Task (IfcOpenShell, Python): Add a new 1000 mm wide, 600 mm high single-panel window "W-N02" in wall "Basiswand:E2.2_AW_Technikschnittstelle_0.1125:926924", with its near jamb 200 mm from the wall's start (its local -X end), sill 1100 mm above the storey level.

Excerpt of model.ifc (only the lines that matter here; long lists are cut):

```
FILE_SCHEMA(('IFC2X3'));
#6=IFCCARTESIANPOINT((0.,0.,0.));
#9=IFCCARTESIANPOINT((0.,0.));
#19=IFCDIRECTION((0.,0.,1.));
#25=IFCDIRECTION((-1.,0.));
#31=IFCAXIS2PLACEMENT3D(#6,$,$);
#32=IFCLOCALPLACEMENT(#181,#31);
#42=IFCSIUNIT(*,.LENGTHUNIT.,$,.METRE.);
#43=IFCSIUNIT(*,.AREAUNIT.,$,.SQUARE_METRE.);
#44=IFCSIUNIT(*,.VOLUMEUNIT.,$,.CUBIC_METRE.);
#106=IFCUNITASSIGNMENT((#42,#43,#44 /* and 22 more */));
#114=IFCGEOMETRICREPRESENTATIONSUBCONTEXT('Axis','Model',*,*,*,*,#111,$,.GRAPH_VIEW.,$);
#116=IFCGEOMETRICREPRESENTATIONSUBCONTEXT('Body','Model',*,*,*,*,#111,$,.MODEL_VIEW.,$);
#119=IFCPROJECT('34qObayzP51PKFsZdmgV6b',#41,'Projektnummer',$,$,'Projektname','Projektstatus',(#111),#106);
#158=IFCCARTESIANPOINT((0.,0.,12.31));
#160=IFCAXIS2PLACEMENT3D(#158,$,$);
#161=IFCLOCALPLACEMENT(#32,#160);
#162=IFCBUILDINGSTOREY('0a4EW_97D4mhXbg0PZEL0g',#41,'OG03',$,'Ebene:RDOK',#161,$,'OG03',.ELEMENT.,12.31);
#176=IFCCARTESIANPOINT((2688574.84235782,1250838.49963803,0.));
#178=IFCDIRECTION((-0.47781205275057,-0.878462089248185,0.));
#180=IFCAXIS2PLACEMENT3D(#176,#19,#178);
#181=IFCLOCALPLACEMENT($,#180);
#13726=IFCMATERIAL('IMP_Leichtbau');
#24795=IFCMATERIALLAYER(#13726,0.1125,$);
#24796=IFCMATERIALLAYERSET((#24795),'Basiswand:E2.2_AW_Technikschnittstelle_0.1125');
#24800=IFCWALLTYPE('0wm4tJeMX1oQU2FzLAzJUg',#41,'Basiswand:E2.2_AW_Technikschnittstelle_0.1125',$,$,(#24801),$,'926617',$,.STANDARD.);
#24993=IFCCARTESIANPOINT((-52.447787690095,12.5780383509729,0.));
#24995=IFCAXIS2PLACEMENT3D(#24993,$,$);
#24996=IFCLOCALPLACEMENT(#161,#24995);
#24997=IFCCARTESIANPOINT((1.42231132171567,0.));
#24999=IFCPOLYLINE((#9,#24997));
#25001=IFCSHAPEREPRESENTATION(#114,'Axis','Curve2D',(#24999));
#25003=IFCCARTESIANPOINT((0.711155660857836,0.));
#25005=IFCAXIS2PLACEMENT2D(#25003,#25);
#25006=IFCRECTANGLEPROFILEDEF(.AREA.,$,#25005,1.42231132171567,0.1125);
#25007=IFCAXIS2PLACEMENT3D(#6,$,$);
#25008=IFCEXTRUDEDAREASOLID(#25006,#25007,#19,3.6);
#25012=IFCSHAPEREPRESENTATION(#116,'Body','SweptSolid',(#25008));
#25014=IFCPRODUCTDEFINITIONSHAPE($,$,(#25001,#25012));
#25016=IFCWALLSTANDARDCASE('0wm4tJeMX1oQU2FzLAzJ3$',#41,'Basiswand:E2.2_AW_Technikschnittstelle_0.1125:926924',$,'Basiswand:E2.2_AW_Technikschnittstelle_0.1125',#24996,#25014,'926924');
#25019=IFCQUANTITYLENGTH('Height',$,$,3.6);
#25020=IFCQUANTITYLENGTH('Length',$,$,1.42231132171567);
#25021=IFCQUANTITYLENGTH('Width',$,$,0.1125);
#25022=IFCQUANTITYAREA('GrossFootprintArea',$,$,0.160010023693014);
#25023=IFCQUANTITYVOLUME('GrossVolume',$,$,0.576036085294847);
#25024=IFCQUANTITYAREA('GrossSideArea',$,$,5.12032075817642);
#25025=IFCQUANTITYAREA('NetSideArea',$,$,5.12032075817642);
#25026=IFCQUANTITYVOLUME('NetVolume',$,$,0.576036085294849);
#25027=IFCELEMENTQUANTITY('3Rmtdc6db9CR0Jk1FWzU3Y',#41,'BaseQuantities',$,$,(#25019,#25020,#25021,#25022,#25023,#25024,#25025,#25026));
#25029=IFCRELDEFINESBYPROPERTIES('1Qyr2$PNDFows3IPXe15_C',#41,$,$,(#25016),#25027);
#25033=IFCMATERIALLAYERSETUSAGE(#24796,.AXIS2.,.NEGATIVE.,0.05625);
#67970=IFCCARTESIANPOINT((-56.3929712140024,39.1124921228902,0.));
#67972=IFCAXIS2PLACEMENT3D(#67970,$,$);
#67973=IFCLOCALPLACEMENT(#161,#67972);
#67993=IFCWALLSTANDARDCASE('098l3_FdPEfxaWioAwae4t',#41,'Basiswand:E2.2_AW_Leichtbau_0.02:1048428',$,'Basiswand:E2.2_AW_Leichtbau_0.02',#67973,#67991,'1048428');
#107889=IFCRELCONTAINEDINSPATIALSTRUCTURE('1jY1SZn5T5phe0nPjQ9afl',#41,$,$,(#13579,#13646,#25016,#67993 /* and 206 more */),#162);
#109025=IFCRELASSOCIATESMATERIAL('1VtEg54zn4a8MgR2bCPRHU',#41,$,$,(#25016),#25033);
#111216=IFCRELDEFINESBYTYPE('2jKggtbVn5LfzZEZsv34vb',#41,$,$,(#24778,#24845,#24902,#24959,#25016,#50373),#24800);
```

```python
import numpy as np
import ifcopenshell
import ifcopenshell.api.feature
import ifcopenshell.api.geometry
import ifcopenshell.api.pset
import ifcopenshell.api.root
import ifcopenshell.api.spatial
import ifcopenshell.api.type
import ifcopenshell.geom
import ifcopenshell.util.element
import ifcopenshell.util.placement
import ifcopenshell.util.representation
import ifcopenshell.util.shape
import ifcopenshell.util.unit

model = ifcopenshell.open("model.ifc")
unit_scale = ifcopenshell.util.unit.calculate_unit_scale(model)
area_scale = ifcopenshell.util.unit.calculate_unit_scale(model, "AREAUNIT")
volume_scale = ifcopenshell.util.unit.calculate_unit_scale(model, "VOLUMEUNIT")
settings = ifcopenshell.geom.settings()


def volume(element):
    """Net volume in cubic metres, openings subtracted."""
    shape = ifcopenshell.geom.create_shape(settings, element)
    return ifcopenshell.util.shape.get_volume(shape.geometry)


wall = model.by_guid("0wm4tJeMX1oQU2FzLAzJ3$")
storey = ifcopenshell.util.element.get_container(wall, ifc_class="IfcBuildingStorey")
context = ifcopenshell.util.representation.get_context(model, "Model", "Body", "MODEL_VIEW")
before = volume(wall)

width, height, from_end, sill = 1, 0.6, 0.2, 1.1  # metres

# The wall runs along its own X axis, and the end named is its -X end.
wall_shape = ifcopenshell.geom.create_shape(settings, wall)
x, y, z = ifcopenshell.util.shape.get_vertices(wall_shape.geometry).T
start = x.min() + from_end
face, thickness = float(y.min()), float(y.max() - y.min())
wall_matrix = ifcopenshell.util.placement.get_local_placement(wall.ObjectPlacement)
level = ifcopenshell.util.placement.get_local_placement(storey.ObjectPlacement)[2, 3]


def in_wall(x, y):
    """Placement at x, y metres in the wall's axes, at sill height."""
    matrix = wall_matrix.copy()
    matrix[:, 3] = wall_matrix @ np.array([x / unit_scale, y / unit_scale, 0.0, 1.0])
    matrix[2, 3] = level + sill / unit_scale
    return matrix


# Opening: a box that overshoots both wall faces by 50 mm.
opening = ifcopenshell.api.root.create_entity(model, ifc_class="IfcOpeningElement")
box = ifcopenshell.api.geometry.add_wall_representation(
    model, context=context, length=width, height=height, thickness=thickness + 0.1
)
ifcopenshell.api.geometry.assign_representation(model, product=opening, representation=box)
ifcopenshell.api.geometry.edit_object_placement(model, product=opening, matrix=in_wall(start, face - 0.05), is_si=False)
ifcopenshell.api.feature.add_feature(model, feature=opening, element=wall)

window = ifcopenshell.api.root.create_entity(model, ifc_class="IfcWindow", name="W-N02")
window.OverallWidth, window.OverallHeight = width / unit_scale, height / unit_scale
body = ifcopenshell.api.geometry.add_window_representation(
    model,
    context=context,
    overall_width=window.OverallWidth,
    overall_height=window.OverallHeight,
    partition_type="SINGLE_PANEL",
)
ifcopenshell.api.geometry.assign_representation(model, product=window, representation=body)
ifcopenshell.api.spatial.assign_container(model, products=[window], relating_structure=storey)
fills = ifcopenshell.api.feature.add_filling(model, opening=opening, element=window)
fills.OwnerHistory = window.OwnerHistory  # required in IFC2X3

# IFC2X3 keeps the operation on the window style.
style = ifcopenshell.api.root.create_entity(model, ifc_class="IfcWindowStyle", name="W-N02")
style.OperationType, style.ConstructionType = "SINGLE_PANEL", "NOTDEFINED"
style.ParameterTakesPrecedence = style.Sizeable = False
ifcopenshell.api.type.assign_type(model, related_objects=[window], relating_type=style)

# Centre the window in the wall's thickness.
ifcopenshell.api.geometry.edit_object_placement(model, product=window, matrix=in_wall(start, face), is_si=False)
window_shape = ifcopenshell.geom.create_shape(settings, window)
depth = ifcopenshell.util.shape.get_vertices(window_shape.geometry)[:, 1]
offset = face + thickness / 2 - (depth.min() + depth.max()) / 2
ifcopenshell.api.geometry.edit_object_placement(model, product=window, matrix=in_wall(start, offset), is_si=False)

after = volume(wall)

# Update the wall's stored quantities.
qto = model.by_id(ifcopenshell.util.element.get_pset(wall, "BaseQuantities", should_inherit=False)["id"])
ifcopenshell.api.pset.edit_qto(model, qto=qto, properties={
    "NetSideArea": after / thickness / area_scale,
    "NetVolume": after / volume_scale,
})

print(f"wall volume {before:.3f} -> {after:.3f} m3")

model.write("model_rev.ifc")
```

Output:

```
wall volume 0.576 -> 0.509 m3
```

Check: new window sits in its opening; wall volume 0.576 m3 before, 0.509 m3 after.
